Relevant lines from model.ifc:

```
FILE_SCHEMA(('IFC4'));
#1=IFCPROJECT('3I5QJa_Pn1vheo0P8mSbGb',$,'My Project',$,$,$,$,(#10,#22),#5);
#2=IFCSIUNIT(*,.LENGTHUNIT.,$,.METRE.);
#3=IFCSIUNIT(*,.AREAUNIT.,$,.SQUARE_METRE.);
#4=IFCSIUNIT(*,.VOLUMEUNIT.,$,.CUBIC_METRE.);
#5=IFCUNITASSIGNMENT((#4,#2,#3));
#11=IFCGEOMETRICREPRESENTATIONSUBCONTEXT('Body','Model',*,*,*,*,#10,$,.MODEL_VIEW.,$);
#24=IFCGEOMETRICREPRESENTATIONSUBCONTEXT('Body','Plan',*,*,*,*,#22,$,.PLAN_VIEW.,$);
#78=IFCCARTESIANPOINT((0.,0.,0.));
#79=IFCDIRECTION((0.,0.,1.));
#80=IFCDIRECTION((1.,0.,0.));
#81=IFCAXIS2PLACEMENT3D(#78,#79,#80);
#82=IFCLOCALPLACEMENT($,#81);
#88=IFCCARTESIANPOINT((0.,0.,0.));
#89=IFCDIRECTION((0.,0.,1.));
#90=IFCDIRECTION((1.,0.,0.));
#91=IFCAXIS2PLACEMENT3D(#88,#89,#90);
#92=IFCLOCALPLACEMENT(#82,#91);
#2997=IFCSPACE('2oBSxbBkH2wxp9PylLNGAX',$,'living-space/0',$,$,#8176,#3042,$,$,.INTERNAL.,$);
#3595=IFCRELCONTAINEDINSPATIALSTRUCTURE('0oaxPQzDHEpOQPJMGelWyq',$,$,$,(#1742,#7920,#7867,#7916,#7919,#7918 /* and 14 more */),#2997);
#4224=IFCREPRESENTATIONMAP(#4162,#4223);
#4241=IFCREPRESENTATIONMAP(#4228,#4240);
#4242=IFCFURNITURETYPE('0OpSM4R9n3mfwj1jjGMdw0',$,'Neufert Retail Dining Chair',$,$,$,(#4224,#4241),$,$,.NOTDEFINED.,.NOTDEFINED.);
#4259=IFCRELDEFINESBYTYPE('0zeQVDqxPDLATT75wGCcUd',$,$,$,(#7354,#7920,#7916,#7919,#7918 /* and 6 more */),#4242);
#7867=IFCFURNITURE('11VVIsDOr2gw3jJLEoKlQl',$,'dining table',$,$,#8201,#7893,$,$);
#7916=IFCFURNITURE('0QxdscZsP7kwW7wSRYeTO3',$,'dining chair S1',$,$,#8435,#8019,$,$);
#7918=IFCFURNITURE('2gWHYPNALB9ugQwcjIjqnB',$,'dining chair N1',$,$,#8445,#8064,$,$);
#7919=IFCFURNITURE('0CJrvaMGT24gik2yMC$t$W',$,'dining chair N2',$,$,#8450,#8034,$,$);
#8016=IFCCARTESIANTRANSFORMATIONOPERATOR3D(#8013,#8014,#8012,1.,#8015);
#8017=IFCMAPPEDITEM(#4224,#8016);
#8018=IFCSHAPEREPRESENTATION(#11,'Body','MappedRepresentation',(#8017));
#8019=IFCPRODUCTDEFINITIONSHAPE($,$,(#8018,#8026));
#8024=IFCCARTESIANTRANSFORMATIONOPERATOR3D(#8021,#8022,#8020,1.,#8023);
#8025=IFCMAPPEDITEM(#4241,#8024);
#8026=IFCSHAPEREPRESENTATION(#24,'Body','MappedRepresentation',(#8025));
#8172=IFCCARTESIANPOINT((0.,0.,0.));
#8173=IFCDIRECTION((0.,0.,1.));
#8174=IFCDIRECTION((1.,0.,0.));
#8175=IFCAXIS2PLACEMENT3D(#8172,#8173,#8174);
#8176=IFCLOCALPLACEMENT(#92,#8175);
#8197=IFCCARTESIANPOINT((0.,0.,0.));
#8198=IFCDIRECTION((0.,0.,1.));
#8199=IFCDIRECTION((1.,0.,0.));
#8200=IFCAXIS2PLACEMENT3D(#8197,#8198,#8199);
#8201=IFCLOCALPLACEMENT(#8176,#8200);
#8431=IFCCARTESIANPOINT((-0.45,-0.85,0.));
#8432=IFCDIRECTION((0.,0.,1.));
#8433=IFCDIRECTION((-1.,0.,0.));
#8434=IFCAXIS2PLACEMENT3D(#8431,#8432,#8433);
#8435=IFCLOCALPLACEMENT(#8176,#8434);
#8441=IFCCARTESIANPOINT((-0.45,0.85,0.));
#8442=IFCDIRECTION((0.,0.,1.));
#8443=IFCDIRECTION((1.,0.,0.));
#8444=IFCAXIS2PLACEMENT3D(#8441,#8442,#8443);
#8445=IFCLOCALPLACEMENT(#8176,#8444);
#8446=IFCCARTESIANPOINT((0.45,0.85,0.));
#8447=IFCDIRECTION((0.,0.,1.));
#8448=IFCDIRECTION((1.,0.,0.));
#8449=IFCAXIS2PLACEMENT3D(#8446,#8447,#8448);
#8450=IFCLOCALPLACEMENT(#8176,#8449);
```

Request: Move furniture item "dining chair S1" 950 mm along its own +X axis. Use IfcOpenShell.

```python
import ifcopenshell
import ifcopenshell.api.geometry
import ifcopenshell.util.placement
import ifcopenshell.util.unit

model = ifcopenshell.open("model.ifc")
unit_scale = ifcopenshell.util.unit.calculate_unit_scale(model)

item = model.by_id(7916)
matrix = ifcopenshell.util.placement.get_local_placement(item.ObjectPlacement)
matrix[:3, 3] += matrix[:3, 0] * 0.95 / unit_scale
ifcopenshell.api.geometry.edit_object_placement(model, product=item, matrix=matrix, is_si=False)

print(ifcopenshell.util.placement.get_local_placement(item.ObjectPlacement).round(3) + 0.0)

model.write("model_rev.ifc")
```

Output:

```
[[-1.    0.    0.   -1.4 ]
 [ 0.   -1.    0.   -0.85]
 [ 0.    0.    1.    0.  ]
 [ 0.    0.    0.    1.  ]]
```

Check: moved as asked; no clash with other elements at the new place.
